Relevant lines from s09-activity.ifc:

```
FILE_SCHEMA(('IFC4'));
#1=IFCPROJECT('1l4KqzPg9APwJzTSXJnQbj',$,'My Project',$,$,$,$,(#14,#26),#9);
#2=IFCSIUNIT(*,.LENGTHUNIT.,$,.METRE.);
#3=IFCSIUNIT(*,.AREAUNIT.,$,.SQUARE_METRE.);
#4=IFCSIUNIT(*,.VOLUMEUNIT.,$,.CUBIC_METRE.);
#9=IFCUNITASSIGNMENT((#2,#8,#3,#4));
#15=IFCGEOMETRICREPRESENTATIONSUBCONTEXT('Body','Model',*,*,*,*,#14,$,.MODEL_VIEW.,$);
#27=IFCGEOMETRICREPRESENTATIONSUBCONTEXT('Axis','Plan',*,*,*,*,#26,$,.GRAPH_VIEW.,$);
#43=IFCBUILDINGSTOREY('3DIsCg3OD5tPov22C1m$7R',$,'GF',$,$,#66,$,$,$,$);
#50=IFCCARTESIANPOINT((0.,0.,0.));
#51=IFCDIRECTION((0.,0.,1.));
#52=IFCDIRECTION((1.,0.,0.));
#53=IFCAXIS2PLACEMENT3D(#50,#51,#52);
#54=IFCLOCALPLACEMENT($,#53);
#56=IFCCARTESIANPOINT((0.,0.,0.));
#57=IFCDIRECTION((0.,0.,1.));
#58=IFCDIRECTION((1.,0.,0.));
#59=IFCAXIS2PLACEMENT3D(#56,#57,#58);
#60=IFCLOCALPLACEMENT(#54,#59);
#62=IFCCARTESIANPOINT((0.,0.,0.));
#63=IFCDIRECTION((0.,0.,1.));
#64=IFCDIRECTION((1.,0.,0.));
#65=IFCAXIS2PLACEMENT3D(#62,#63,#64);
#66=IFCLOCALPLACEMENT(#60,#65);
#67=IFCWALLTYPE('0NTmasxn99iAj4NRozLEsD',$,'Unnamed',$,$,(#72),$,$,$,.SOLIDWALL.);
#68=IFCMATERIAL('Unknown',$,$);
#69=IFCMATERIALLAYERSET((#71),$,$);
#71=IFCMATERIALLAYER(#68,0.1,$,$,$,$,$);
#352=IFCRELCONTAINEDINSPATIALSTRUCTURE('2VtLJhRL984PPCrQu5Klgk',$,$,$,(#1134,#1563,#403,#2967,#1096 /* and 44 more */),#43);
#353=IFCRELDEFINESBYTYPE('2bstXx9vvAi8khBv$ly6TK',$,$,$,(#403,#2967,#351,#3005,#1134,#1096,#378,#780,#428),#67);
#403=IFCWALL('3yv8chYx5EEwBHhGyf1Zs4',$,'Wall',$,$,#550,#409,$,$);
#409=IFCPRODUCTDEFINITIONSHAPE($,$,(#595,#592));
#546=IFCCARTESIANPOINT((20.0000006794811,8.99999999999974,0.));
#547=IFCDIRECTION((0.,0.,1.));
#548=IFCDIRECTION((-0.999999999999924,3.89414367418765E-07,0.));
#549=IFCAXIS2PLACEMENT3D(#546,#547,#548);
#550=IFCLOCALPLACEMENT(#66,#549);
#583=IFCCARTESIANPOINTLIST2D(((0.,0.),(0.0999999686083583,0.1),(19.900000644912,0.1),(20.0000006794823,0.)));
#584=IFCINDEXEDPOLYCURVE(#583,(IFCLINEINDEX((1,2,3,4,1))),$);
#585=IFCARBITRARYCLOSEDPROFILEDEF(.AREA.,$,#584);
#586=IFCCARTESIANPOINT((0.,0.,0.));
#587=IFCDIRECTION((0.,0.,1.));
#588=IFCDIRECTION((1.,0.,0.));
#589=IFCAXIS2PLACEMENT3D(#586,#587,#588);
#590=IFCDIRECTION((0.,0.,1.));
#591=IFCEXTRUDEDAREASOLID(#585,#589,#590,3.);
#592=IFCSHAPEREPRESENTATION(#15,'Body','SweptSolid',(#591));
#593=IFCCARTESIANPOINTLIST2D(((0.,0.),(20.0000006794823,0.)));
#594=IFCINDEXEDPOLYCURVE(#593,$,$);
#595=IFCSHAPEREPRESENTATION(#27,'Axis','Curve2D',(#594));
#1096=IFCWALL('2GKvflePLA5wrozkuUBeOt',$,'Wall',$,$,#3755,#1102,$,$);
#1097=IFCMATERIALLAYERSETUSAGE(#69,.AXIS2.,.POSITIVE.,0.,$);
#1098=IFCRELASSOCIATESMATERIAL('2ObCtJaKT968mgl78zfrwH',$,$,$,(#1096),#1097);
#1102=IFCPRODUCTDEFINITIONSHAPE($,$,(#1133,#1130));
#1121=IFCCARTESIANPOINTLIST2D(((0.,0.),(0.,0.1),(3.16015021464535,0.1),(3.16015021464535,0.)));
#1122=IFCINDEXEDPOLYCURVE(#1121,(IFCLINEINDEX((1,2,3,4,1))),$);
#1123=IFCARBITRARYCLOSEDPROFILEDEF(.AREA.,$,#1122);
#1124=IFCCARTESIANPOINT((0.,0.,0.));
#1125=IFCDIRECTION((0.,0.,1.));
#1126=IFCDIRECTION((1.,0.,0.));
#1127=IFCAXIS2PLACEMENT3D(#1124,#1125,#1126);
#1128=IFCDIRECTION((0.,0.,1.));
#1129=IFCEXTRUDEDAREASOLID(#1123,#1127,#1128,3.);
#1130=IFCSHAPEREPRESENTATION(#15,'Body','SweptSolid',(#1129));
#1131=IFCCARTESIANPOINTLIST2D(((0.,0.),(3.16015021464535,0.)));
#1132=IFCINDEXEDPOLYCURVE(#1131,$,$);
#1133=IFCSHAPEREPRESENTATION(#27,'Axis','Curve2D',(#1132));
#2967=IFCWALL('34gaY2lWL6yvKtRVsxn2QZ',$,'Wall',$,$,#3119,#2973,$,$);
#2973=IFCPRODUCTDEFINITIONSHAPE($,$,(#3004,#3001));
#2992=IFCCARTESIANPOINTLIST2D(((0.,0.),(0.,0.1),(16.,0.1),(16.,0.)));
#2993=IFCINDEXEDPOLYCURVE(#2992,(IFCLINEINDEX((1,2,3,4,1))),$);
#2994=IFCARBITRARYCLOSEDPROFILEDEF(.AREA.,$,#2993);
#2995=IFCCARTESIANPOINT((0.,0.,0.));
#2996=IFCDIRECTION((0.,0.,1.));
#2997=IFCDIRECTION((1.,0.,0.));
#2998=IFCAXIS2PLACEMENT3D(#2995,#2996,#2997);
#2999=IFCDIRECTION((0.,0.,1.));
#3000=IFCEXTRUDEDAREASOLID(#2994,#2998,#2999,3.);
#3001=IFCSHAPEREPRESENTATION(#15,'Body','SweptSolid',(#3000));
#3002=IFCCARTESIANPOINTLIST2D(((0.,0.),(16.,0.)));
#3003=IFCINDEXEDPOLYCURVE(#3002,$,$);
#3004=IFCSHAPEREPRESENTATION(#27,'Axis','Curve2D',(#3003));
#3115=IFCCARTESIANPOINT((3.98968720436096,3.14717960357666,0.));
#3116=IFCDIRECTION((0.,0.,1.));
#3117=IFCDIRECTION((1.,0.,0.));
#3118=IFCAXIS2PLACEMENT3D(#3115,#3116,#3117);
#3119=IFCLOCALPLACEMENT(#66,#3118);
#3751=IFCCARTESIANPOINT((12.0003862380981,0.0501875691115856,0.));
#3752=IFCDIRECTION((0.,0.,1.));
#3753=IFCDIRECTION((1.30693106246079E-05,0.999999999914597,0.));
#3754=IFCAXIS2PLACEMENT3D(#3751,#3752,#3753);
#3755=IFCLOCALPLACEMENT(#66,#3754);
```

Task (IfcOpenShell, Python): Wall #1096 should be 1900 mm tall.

```python
import ifcopenshell
import ifcopenshell.geom
import ifcopenshell.util.representation
import ifcopenshell.util.shape

model = ifcopenshell.open("s09-activity.ifc")
settings = ifcopenshell.geom.settings()


def volume(element):
    """Net volume in cubic metres, openings subtracted."""
    shape = ifcopenshell.geom.create_shape(settings, element)
    return ifcopenshell.util.shape.get_volume(shape.geometry)


wall = model.by_guid("2GKvflePLA5wrozkuUBeOt")
before = volume(wall)

body = ifcopenshell.util.representation.get_representation(wall, "Model", "Body")
solid = body.Items[0]
old_height = solid.Depth
solid.Depth = 1.9
after = volume(wall)

print(f"height {old_height:g} -> {solid.Depth:g}, volume {before:.3f} -> {after:.3f} m3")

model.write("s09-activity_edited.ifc")
```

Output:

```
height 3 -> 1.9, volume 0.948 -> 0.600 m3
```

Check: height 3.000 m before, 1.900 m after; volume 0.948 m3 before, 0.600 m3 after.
